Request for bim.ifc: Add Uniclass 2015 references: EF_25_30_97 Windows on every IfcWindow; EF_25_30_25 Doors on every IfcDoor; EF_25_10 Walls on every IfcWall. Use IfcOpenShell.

First a look at what the model holds.

```python
import ifcopenshell

model = ifcopenshell.open("bim.ifc")
print(model.schema)
print("classifications:", [c.Name for c in model.by_type("IfcClassification")])
for ifc_class in ("IfcDoor", "IfcRoof", "IfcStair", "IfcWall", "IfcWindow"):
    print(ifc_class, len(model.by_type(ifc_class)))
```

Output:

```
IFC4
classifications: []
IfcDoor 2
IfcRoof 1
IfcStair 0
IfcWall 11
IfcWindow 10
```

```python
import ifcopenshell
import ifcopenshell.api.classification

model = ifcopenshell.open("bim.ifc")

system = ifcopenshell.api.classification.add_classification(model, classification="Uniclass 2015")

codes = {
    "IfcWindow": ("EF_25_30_97", "Windows"),
    "IfcDoor": ("EF_25_30_25", "Doors"),
    "IfcWall": ("EF_25_10", "Walls"),
}
for ifc_class, (code, name) in codes.items():
    products = model.by_type(ifc_class)
    ifcopenshell.api.classification.add_reference(
        model, products=products, classification=system, identification=code, name=name
    )
    print(code, len(products))

model.write("bim_rev.ifc")
```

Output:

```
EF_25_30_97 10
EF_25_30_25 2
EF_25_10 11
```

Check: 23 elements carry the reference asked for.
